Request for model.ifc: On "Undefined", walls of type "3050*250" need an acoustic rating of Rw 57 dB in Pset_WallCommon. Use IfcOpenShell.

First a look at what the model holds.

```python
import ifcopenshell
import ifcopenshell.util.element

model = ifcopenshell.open("model.ifc")
print(model.schema)
storey = next(s for s in model.by_type("IfcBuildingStorey") if s.Name == "Undefined")
walls = [e for e in ifcopenshell.util.element.get_decomposition(storey) if e.is_a("IfcWall")]
seen = {}
for e in walls:
    element_type = ifcopenshell.util.element.get_type(e)
    key = (element_type.Name if element_type != e and element_type else None, ifcopenshell.util.element.get_pset(e, "Pset_WallCommon", "AcousticRating"))
    seen[key] = seen.get(key, 0) + 1
for (name, value), count in sorted(seen.items(), key=str):
    print(count, "x", name, "|", value)
```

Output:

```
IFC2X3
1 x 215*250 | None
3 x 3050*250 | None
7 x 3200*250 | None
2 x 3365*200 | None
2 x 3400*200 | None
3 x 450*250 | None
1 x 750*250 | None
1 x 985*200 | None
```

```python
import ifcopenshell
import ifcopenshell.api.pset
import ifcopenshell.util.element

model = ifcopenshell.open("model.ifc")

storey = next(s for s in model.by_type("IfcBuildingStorey") if s.Name == "Undefined")
walls = [e for e in ifcopenshell.util.element.get_decomposition(storey) if e.is_a("IfcWall")]

count = 0
for e in walls:
    element_type = ifcopenshell.util.element.get_type(e)
    if element_type in (None, e) or element_type.Name != "3050*250":
        continue
    # add_pset returns the element's existing set when there is one.
    pset = ifcopenshell.api.pset.add_pset(model, product=e, name="Pset_WallCommon")
    ifcopenshell.api.pset.edit_pset(model, pset=pset, properties={"AcousticRating": "Rw 57 dB"})
    count += 1

print(count, "walls updated")

model.write("model_v2.ifc")
```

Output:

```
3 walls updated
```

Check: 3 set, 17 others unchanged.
